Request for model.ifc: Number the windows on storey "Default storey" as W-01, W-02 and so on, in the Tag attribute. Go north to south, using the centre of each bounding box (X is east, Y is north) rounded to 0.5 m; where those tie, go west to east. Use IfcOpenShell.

First a look at what the model holds.

```python
import ifcopenshell
import ifcopenshell.util.element
import ifcopenshell.util.placement

model = ifcopenshell.open("model.ifc")
print(model.schema)
storey = next(s for s in model.by_type("IfcBuildingStorey") if s.Name == "Default storey")
windows = [e for e in ifcopenshell.util.element.get_decomposition(storey) if e.is_a("IfcWindow")]
for e in sorted(windows, key=lambda e: e.id()):
    origin = ifcopenshell.util.placement.get_local_placement(e.ObjectPlacement)[:3, 3]
    print(e.id(), e.Tag, e.Name, origin.round(2) + 0.0, sep=" | ")
```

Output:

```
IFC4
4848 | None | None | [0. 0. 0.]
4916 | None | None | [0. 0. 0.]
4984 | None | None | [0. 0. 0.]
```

```python
import ifcopenshell
import ifcopenshell.geom
import ifcopenshell.util.element
import ifcopenshell.util.shape

model = ifcopenshell.open("model.ifc")
settings = ifcopenshell.geom.settings()
settings.set("use-world-coords", True)


def centre(element):
    shape = ifcopenshell.geom.create_shape(settings, element)
    return ifcopenshell.util.shape.get_bbox_centroid(shape.geometry)


storey = next(s for s in model.by_type("IfcBuildingStorey") if s.Name == "Default storey")
windows = [e for e in ifcopenshell.util.element.get_decomposition(storey) if e.is_a("IfcWindow")]

# Insertion points can sit at a corner or the storey origin, so sort by the geometry (in metres).
centres = {e: centre(e) for e in windows}
windows.sort(key=lambda e: (-round(centres[e][1] / 0.5), centres[e][0]))

for i, e in enumerate(windows, start=1):
    number = f"W-{i:02d}"
    e.Tag = number
    print(e.id(), number)

model.write("model_edited.ifc")
```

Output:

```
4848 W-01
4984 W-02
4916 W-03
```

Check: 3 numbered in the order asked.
